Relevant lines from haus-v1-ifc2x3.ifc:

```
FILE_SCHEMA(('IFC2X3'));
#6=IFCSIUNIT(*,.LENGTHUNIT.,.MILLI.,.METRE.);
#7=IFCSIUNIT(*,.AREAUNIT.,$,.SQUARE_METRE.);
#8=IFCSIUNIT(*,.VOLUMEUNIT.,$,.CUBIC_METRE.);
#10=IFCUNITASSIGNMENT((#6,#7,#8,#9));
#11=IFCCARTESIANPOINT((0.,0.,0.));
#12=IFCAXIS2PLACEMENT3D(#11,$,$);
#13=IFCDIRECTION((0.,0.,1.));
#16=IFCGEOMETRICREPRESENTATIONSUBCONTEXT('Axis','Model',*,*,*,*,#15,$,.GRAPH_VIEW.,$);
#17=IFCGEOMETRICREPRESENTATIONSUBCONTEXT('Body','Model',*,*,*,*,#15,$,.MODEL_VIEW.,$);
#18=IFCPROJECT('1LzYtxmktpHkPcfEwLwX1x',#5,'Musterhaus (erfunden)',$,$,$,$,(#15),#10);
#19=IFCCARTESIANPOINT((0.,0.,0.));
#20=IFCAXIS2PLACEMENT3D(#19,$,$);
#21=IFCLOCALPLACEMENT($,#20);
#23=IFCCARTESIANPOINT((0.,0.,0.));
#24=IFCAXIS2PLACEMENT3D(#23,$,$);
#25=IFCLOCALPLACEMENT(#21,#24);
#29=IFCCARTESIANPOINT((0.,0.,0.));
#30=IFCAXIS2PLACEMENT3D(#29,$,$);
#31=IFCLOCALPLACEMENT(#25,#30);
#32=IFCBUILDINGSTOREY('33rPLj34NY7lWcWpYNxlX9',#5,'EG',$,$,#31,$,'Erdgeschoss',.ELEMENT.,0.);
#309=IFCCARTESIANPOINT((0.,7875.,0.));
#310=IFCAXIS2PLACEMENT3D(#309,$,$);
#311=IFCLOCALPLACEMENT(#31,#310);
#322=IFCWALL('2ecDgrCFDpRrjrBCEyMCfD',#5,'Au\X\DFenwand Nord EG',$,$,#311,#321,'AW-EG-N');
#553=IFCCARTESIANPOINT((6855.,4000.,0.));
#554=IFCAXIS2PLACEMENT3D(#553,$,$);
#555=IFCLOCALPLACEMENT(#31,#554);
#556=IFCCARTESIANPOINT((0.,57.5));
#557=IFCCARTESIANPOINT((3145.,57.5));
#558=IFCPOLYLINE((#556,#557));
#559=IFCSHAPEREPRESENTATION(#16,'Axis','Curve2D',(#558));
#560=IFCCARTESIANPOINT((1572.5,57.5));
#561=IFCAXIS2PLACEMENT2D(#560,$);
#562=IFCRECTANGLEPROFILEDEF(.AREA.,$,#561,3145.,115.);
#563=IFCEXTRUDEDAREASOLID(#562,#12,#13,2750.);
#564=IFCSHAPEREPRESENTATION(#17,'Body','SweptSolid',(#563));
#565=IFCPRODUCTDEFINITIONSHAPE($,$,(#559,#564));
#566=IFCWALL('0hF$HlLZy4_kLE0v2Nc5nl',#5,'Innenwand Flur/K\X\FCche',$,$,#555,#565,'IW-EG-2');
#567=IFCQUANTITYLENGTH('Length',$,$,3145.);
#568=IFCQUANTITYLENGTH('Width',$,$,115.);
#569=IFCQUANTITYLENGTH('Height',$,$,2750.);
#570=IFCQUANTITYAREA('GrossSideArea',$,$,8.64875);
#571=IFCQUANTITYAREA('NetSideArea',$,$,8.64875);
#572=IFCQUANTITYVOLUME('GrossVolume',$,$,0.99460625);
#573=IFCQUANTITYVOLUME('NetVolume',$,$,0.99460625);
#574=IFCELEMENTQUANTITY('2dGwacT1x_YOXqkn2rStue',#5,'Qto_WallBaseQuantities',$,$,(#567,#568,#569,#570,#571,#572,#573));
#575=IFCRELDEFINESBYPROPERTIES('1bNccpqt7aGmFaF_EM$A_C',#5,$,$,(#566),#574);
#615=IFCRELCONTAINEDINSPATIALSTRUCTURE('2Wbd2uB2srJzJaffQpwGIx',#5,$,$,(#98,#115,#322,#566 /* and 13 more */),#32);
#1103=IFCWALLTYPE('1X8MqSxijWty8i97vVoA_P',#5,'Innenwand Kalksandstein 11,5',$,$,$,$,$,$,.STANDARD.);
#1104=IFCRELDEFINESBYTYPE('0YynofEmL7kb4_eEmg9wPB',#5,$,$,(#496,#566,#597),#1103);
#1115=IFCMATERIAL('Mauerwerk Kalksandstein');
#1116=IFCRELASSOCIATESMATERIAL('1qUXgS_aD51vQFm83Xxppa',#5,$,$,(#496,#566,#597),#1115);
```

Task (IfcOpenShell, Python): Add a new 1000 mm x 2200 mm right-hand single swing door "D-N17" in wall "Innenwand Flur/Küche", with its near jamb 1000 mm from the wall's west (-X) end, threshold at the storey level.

```python
import numpy as np
import ifcopenshell
import ifcopenshell.api.feature
import ifcopenshell.api.geometry
import ifcopenshell.api.pset
import ifcopenshell.api.root
import ifcopenshell.api.spatial
import ifcopenshell.api.type
import ifcopenshell.geom
import ifcopenshell.util.element
import ifcopenshell.util.placement
import ifcopenshell.util.representation
import ifcopenshell.util.shape
import ifcopenshell.util.unit

model = ifcopenshell.open("haus-v1-ifc2x3.ifc")
unit_scale = ifcopenshell.util.unit.calculate_unit_scale(model)
area_scale = ifcopenshell.util.unit.calculate_unit_scale(model, "AREAUNIT")
volume_scale = ifcopenshell.util.unit.calculate_unit_scale(model, "VOLUMEUNIT")
settings = ifcopenshell.geom.settings()


def volume(element):
    """Net volume in cubic metres, openings subtracted."""
    shape = ifcopenshell.geom.create_shape(settings, element)
    return ifcopenshell.util.shape.get_volume(shape.geometry)


wall = model.by_guid("0hF$HlLZy4_kLE0v2Nc5nl")
storey = ifcopenshell.util.element.get_container(wall, ifc_class="IfcBuildingStorey")
context = ifcopenshell.util.representation.get_context(model, "Model", "Body", "MODEL_VIEW")
before = volume(wall)

width, height, from_end, sill = 1, 2.2, 1, 0.0  # metres

# The wall runs along its own X axis, and the end named is its -X end.
wall_shape = ifcopenshell.geom.create_shape(settings, wall)
x, y, z = ifcopenshell.util.shape.get_vertices(wall_shape.geometry).T
start = x.min() + from_end
face, thickness = float(y.min()), float(y.max() - y.min())
wall_matrix = ifcopenshell.util.placement.get_local_placement(wall.ObjectPlacement)
level = ifcopenshell.util.placement.get_local_placement(storey.ObjectPlacement)[2, 3]


def in_wall(x, y):
    """Placement at x, y metres in the wall's axes, at sill height."""
    matrix = wall_matrix.copy()
    matrix[:, 3] = wall_matrix @ np.array([x / unit_scale, y / unit_scale, 0.0, 1.0])
    matrix[2, 3] = level + sill / unit_scale
    return matrix


# Opening: a box that overshoots both wall faces by 50 mm.
opening = ifcopenshell.api.root.create_entity(model, ifc_class="IfcOpeningElement")
box = ifcopenshell.api.geometry.add_wall_representation(
    model, context=context, length=width, height=height, thickness=thickness + 0.1
)
ifcopenshell.api.geometry.assign_representation(model, product=opening, representation=box)
ifcopenshell.api.geometry.edit_object_placement(model, product=opening, matrix=in_wall(start, face - 0.05), is_si=False)
ifcopenshell.api.feature.add_feature(model, feature=opening, element=wall)

door = ifcopenshell.api.root.create_entity(model, ifc_class="IfcDoor", name="D-N17")
door.OverallWidth, door.OverallHeight = width / unit_scale, height / unit_scale
body = ifcopenshell.api.geometry.add_door_representation(
    model,
    context=context,
    overall_width=door.OverallWidth,
    overall_height=door.OverallHeight,
    operation_type="SINGLE_SWING_RIGHT",
    lining_properties={"LiningDepth": thickness / unit_scale, "ThresholdDepth": thickness / unit_scale},
)
ifcopenshell.api.geometry.assign_representation(model, product=door, representation=body)
ifcopenshell.api.spatial.assign_container(model, products=[door], relating_structure=storey)
fills = ifcopenshell.api.feature.add_filling(model, opening=opening, element=door)
fills.OwnerHistory = door.OwnerHistory  # required in IFC2X3

# IFC2X3 keeps the operation on the door style.
style = ifcopenshell.api.root.create_entity(model, ifc_class="IfcDoorStyle", name="D-N17")
style.OperationType, style.ConstructionType = "SINGLE_SWING_RIGHT", "NOTDEFINED"
style.ParameterTakesPrecedence = style.Sizeable = False
ifcopenshell.api.type.assign_type(model, related_objects=[door], relating_type=style)

# The lining spans the wall, so the door starts at the wall face.
ifcopenshell.api.geometry.edit_object_placement(model, product=door, matrix=in_wall(start, face), is_si=False)

after = volume(wall)

# Update the wall's stored quantities.
qto = model.by_id(ifcopenshell.util.element.get_pset(wall, "Qto_WallBaseQuantities", should_inherit=False)["id"])
ifcopenshell.api.pset.edit_qto(model, qto=qto, properties={
    "NetSideArea": after / thickness / area_scale,
    "NetVolume": after / volume_scale,
})

print(f"wall volume {before:.3f} -> {after:.3f} m3")

model.write("haus-v1-ifc2x3-out.ifc")
```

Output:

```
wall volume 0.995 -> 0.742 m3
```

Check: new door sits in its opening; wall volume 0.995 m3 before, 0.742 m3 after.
